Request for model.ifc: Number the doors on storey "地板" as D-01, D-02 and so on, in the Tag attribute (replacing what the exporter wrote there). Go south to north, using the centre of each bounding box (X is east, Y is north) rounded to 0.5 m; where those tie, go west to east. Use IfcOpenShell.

First a look at what the model holds.

```python
import ifcopenshell
import ifcopenshell.util.element
import ifcopenshell.util.placement

model = ifcopenshell.open("model.ifc")
print(model.schema)
storey = next(s for s in model.by_type("IfcBuildingStorey") if s.Name == "地板")
doors = [e for e in ifcopenshell.util.element.get_decomposition(storey) if e.is_a("IfcDoor")]
for e in sorted(doors, key=lambda e: e.id()):
    origin = ifcopenshell.util.placement.get_local_placement(e.ObjectPlacement)[:3, 3]
    print(e.id(), e.Tag, e.Name, origin.round(2) + 0.0, sep=" | ")
```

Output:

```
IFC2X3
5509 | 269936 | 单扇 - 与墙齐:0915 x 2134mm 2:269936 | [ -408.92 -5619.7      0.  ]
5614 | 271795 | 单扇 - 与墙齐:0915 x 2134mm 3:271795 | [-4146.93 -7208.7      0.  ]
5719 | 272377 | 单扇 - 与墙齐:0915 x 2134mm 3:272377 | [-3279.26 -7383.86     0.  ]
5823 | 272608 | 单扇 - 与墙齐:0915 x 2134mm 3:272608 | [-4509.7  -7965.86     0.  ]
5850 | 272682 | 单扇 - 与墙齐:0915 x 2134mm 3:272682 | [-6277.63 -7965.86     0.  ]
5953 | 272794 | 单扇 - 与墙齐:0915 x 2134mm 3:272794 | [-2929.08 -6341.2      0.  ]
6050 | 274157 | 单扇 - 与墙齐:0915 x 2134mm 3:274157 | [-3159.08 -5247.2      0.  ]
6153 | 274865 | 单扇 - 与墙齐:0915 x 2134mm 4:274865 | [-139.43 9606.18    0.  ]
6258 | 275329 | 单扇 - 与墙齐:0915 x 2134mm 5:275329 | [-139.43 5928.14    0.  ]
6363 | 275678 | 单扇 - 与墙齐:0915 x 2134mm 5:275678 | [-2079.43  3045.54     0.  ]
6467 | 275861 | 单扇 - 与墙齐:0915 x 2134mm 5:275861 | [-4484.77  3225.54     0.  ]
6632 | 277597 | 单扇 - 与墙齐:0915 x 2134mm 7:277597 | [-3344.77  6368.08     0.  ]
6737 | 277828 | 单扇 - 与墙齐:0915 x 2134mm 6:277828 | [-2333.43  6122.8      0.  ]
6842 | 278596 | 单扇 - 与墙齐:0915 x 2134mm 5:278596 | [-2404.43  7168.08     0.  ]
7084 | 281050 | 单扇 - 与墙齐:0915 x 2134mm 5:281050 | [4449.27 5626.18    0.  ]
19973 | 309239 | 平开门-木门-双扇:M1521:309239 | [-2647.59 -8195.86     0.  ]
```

```python
import ifcopenshell
import ifcopenshell.geom
import ifcopenshell.util.element
import ifcopenshell.util.shape

model = ifcopenshell.open("model.ifc")
settings = ifcopenshell.geom.settings()
settings.set("use-world-coords", True)


def centre(element):
    shape = ifcopenshell.geom.create_shape(settings, element)
    return ifcopenshell.util.shape.get_bbox_centroid(shape.geometry)


storey = next(s for s in model.by_type("IfcBuildingStorey") if s.Name == "地板")
doors = [e for e in ifcopenshell.util.element.get_decomposition(storey) if e.is_a("IfcDoor")]

# Insertion points can sit at a corner or the storey origin, so sort by the geometry (in metres).
centres = {e: centre(e) for e in doors}
doors.sort(key=lambda e: (round(centres[e][1] / 0.5), centres[e][0]))

for i, e in enumerate(doors, start=1):
    number = f"D-{i:02d}"
    e.Tag = number
    print(e.id(), number)

model.write("model_updated.ifc")
```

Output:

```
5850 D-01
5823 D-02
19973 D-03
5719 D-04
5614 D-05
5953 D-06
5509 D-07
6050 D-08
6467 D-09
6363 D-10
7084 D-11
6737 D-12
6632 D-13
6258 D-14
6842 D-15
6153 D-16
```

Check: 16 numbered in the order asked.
